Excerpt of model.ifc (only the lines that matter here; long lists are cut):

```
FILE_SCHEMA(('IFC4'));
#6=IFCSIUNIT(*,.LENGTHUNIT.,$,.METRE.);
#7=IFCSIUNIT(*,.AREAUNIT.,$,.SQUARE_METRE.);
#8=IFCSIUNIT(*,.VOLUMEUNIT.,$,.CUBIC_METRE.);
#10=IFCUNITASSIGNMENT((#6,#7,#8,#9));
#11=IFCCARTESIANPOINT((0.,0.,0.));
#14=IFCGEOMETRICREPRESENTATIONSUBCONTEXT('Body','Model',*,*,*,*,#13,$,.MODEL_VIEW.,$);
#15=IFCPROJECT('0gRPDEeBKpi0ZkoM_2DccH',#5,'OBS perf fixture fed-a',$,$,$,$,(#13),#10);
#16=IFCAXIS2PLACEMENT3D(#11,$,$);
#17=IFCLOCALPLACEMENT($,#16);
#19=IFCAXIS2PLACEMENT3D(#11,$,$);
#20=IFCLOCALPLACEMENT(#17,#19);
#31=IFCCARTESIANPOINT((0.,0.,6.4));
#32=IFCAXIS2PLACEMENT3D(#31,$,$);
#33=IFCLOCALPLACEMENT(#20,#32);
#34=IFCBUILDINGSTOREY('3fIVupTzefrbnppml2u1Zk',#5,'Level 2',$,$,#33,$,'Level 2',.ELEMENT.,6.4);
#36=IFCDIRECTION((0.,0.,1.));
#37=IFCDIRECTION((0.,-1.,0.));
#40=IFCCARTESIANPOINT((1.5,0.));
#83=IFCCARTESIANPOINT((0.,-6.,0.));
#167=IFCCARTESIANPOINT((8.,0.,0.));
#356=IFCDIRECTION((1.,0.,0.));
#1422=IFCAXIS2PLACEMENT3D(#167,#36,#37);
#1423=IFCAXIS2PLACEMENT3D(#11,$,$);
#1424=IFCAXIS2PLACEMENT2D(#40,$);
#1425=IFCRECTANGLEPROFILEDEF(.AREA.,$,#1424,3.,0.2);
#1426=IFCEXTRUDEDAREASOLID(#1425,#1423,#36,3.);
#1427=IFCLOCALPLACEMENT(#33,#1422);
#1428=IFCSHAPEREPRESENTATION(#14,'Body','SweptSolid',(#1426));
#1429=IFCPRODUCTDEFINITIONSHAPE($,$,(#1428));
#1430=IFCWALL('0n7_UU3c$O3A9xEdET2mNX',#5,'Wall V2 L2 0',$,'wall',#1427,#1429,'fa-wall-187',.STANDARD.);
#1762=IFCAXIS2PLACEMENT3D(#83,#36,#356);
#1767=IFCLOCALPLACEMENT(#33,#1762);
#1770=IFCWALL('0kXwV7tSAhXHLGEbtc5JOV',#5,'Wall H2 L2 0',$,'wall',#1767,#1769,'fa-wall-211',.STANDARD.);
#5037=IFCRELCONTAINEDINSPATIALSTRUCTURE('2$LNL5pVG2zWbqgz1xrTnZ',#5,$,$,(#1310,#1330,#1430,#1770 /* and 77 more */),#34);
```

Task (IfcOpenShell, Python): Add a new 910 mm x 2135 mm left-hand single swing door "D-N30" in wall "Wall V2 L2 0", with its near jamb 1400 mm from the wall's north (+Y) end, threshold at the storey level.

```python
import numpy as np
import ifcopenshell
import ifcopenshell.api.feature
import ifcopenshell.api.geometry
import ifcopenshell.api.root
import ifcopenshell.api.spatial
import ifcopenshell.geom
import ifcopenshell.util.element
import ifcopenshell.util.placement
import ifcopenshell.util.representation
import ifcopenshell.util.shape
import ifcopenshell.util.unit

model = ifcopenshell.open("model.ifc")
unit_scale = ifcopenshell.util.unit.calculate_unit_scale(model)
settings = ifcopenshell.geom.settings()


def volume(element):
    """Net volume in cubic metres, openings subtracted."""
    shape = ifcopenshell.geom.create_shape(settings, element)
    return ifcopenshell.util.shape.get_volume(shape.geometry)


wall = model.by_guid("0n7_UU3c$O3A9xEdET2mNX")
storey = ifcopenshell.util.element.get_container(wall, ifc_class="IfcBuildingStorey")
context = ifcopenshell.util.representation.get_context(model, "Model", "Body", "MODEL_VIEW")
before = volume(wall)

width, height, from_end, sill = 0.91, 2.135, 1.4, 0.0  # metres

# The wall runs along its own X axis, and the end named is its -X end.
wall_shape = ifcopenshell.geom.create_shape(settings, wall)
x, y, z = ifcopenshell.util.shape.get_vertices(wall_shape.geometry).T
start = x.min() + from_end
face, thickness = float(y.min()), float(y.max() - y.min())
wall_matrix = ifcopenshell.util.placement.get_local_placement(wall.ObjectPlacement)
level = ifcopenshell.util.placement.get_local_placement(storey.ObjectPlacement)[2, 3]


def in_wall(x, y):
    """Placement at x, y metres in the wall's axes, at sill height."""
    matrix = wall_matrix.copy()
    matrix[:, 3] = wall_matrix @ np.array([x / unit_scale, y / unit_scale, 0.0, 1.0])
    matrix[2, 3] = level + sill / unit_scale
    return matrix


# Opening: a box that overshoots both wall faces by 50 mm.
opening = ifcopenshell.api.root.create_entity(model, ifc_class="IfcOpeningElement", predefined_type="OPENING")
box = ifcopenshell.api.geometry.add_wall_representation(
    model, context=context, length=width, height=height, thickness=thickness + 0.1
)
ifcopenshell.api.geometry.assign_representation(model, product=opening, representation=box)
ifcopenshell.api.geometry.edit_object_placement(model, product=opening, matrix=in_wall(start, face - 0.05), is_si=False)
ifcopenshell.api.feature.add_feature(model, feature=opening, element=wall)

door = ifcopenshell.api.root.create_entity(model, ifc_class="IfcDoor", name="D-N30", predefined_type="DOOR")
door.OverallWidth, door.OverallHeight = width / unit_scale, height / unit_scale
door.OperationType = "SINGLE_SWING_LEFT"
body = ifcopenshell.api.geometry.add_door_representation(
    model,
    context=context,
    overall_width=door.OverallWidth,
    overall_height=door.OverallHeight,
    operation_type="SINGLE_SWING_LEFT",
    lining_properties={"LiningDepth": thickness / unit_scale, "ThresholdDepth": thickness / unit_scale},
)
ifcopenshell.api.geometry.assign_representation(model, product=door, representation=body)
ifcopenshell.api.spatial.assign_container(model, products=[door], relating_structure=storey)
ifcopenshell.api.feature.add_filling(model, opening=opening, element=door)

# The lining spans the wall, so the door starts at the wall face.
ifcopenshell.api.geometry.edit_object_placement(model, product=door, matrix=in_wall(start, face), is_si=False)

after = volume(wall)

print(f"wall volume {before:.3f} -> {after:.3f} m3")

model.write("model_v2.ifc")
```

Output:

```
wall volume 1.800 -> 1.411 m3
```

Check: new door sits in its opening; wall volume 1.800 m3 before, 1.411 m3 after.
